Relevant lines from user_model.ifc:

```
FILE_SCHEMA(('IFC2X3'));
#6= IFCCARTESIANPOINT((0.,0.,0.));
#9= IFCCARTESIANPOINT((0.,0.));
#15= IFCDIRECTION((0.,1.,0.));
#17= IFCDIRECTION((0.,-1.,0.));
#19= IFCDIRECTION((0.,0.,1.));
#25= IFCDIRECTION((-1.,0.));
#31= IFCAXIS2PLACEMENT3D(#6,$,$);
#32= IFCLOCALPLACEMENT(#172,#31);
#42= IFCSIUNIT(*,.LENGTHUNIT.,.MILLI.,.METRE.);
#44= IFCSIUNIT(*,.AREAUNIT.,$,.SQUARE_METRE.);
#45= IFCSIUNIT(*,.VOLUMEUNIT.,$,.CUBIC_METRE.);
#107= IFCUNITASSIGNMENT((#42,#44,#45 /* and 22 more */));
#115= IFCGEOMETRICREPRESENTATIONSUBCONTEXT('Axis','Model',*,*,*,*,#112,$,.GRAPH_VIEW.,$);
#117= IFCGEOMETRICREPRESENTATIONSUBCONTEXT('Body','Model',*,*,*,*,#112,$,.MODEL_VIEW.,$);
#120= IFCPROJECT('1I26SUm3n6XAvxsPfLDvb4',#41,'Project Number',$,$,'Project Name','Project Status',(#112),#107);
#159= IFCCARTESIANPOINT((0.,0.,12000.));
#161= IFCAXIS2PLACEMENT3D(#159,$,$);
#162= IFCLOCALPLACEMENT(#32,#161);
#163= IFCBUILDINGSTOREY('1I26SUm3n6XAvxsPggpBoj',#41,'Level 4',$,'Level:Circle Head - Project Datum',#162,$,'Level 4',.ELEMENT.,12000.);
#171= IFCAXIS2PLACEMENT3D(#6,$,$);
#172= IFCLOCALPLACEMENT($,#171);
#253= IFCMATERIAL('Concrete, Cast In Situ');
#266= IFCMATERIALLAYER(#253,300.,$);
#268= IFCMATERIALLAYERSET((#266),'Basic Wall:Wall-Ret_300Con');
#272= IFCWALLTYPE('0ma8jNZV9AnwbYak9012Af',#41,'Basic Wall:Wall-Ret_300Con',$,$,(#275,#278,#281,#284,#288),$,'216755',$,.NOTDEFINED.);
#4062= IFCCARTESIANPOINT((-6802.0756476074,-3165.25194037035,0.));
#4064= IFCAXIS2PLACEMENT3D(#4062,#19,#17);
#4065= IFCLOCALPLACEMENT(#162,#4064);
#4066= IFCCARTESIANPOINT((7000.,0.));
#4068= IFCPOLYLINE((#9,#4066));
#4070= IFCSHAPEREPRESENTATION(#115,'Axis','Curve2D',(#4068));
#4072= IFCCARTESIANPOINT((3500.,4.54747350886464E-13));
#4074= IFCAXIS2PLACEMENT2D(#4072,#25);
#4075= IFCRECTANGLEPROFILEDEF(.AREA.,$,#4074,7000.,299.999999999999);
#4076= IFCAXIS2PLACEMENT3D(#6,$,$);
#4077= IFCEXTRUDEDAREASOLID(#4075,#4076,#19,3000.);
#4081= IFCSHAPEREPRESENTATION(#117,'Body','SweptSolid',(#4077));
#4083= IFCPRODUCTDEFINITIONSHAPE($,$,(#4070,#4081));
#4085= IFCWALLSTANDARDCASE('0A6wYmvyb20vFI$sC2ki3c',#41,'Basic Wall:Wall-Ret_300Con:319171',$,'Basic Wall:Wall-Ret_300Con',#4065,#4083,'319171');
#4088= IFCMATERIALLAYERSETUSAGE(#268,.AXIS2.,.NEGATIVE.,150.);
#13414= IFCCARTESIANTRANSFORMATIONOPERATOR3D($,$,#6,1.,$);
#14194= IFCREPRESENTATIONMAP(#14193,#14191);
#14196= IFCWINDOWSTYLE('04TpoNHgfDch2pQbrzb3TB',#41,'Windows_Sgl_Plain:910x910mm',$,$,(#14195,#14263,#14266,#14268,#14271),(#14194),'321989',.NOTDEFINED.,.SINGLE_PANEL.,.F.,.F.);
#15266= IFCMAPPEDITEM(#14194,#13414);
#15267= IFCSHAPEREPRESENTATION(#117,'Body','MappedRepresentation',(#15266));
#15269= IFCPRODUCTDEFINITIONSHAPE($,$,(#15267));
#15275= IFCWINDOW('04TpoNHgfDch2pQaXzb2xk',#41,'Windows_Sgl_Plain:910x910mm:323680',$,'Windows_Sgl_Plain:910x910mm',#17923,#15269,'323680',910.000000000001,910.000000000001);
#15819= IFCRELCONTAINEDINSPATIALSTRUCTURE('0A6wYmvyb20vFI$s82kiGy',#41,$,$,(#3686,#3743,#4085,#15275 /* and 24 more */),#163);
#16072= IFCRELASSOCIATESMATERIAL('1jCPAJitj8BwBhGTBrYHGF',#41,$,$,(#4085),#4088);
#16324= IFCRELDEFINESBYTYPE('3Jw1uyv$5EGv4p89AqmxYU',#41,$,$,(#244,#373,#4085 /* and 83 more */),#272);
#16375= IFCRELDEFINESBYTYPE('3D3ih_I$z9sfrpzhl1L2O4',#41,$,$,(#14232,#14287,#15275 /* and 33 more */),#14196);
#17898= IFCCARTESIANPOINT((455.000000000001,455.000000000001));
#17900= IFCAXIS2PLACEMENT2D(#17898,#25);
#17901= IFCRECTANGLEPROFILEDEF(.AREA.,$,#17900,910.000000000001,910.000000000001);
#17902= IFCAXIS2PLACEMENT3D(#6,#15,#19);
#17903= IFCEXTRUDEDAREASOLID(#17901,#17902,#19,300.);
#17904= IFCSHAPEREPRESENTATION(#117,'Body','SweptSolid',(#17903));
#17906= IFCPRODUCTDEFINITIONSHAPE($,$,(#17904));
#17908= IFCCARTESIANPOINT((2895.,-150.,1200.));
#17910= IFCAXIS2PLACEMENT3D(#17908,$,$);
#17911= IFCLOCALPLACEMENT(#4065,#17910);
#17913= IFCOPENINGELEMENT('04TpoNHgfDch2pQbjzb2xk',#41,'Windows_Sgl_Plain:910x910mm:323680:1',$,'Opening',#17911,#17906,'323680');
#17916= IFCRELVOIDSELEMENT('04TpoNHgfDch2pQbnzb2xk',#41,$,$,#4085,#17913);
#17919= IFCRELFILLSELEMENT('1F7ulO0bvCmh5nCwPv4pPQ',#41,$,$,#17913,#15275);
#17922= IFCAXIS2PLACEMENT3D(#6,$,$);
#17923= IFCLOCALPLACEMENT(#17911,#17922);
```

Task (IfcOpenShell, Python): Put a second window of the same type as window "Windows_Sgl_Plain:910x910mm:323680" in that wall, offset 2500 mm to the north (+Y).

```python
import ifcopenshell
import ifcopenshell.api.feature
import ifcopenshell.api.geometry
import ifcopenshell.api.root
import ifcopenshell.geom
import ifcopenshell.util.element
import ifcopenshell.util.placement
import ifcopenshell.util.shape

model = ifcopenshell.open("user_model.ifc")
settings = ifcopenshell.geom.settings()


def volume(element):
    """Net volume in cubic metres, openings subtracted."""
    shape = ifcopenshell.geom.create_shape(settings, element)
    return ifcopenshell.util.shape.get_volume(shape.geometry)


def reuse_history(source, copy):
    """copy_class also copies each property set's owner history, people and application; keep the originals."""
    for rel in copy.IsDefinedBy:
        if rel.is_a("IfcRelDefinesByProperties") and (history := rel.RelatingPropertyDefinition.OwnerHistory):
            rel.RelatingPropertyDefinition.OwnerHistory = source.OwnerHistory
            ifcopenshell.util.element.remove_deep2(model, history)


window = model.by_guid("04TpoNHgfDch2pQaXzb2xk")
opening = window.FillsVoids[0].RelatingOpeningElement
wall = opening.VoidsElements[0].RelatingBuildingElement
before = volume(wall)
shift = ifcopenshell.util.placement.get_local_placement(wall.ObjectPlacement)[:3, 0] * -2500.0

# copy_class copies the void relationship, type, container and properties, but no geometry.
new_opening = ifcopenshell.api.root.copy_class(model, product=opening)
new_opening.Representation = ifcopenshell.util.element.copy_deep(
    model, opening.Representation, exclude=["IfcGeometricRepresentationContext", "IfcRepresentationMap"]
)
new_opening.Name = "Windows_Sgl_Plain:910x910mm"
new_opening.Tag = None
new_window = ifcopenshell.api.root.copy_class(model, product=window)
new_window.Representation = ifcopenshell.util.element.copy_deep(
    model, window.Representation, exclude=["IfcGeometricRepresentationContext", "IfcRepresentationMap"]
)
new_window.Name = "Windows_Sgl_Plain:910x910mm"
new_window.Tag = None
reuse_history(window, new_window)
fills = ifcopenshell.api.feature.add_filling(model, opening=new_opening, element=new_window)
fills.OwnerHistory = new_window.OwnerHistory  # required in IFC2X3

for old, new in ((opening, new_opening), (window, new_window)):
    matrix = ifcopenshell.util.placement.get_local_placement(old.ObjectPlacement)
    matrix[:3, 3] += shift
    ifcopenshell.api.geometry.edit_object_placement(model, product=new, matrix=matrix, is_si=False)

after = volume(wall)

print(f"wall volume {before:.3f} -> {after:.3f} m3")

model.write("user_model-out.ifc")
```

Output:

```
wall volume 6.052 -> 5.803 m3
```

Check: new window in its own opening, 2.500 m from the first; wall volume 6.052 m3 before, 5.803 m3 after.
